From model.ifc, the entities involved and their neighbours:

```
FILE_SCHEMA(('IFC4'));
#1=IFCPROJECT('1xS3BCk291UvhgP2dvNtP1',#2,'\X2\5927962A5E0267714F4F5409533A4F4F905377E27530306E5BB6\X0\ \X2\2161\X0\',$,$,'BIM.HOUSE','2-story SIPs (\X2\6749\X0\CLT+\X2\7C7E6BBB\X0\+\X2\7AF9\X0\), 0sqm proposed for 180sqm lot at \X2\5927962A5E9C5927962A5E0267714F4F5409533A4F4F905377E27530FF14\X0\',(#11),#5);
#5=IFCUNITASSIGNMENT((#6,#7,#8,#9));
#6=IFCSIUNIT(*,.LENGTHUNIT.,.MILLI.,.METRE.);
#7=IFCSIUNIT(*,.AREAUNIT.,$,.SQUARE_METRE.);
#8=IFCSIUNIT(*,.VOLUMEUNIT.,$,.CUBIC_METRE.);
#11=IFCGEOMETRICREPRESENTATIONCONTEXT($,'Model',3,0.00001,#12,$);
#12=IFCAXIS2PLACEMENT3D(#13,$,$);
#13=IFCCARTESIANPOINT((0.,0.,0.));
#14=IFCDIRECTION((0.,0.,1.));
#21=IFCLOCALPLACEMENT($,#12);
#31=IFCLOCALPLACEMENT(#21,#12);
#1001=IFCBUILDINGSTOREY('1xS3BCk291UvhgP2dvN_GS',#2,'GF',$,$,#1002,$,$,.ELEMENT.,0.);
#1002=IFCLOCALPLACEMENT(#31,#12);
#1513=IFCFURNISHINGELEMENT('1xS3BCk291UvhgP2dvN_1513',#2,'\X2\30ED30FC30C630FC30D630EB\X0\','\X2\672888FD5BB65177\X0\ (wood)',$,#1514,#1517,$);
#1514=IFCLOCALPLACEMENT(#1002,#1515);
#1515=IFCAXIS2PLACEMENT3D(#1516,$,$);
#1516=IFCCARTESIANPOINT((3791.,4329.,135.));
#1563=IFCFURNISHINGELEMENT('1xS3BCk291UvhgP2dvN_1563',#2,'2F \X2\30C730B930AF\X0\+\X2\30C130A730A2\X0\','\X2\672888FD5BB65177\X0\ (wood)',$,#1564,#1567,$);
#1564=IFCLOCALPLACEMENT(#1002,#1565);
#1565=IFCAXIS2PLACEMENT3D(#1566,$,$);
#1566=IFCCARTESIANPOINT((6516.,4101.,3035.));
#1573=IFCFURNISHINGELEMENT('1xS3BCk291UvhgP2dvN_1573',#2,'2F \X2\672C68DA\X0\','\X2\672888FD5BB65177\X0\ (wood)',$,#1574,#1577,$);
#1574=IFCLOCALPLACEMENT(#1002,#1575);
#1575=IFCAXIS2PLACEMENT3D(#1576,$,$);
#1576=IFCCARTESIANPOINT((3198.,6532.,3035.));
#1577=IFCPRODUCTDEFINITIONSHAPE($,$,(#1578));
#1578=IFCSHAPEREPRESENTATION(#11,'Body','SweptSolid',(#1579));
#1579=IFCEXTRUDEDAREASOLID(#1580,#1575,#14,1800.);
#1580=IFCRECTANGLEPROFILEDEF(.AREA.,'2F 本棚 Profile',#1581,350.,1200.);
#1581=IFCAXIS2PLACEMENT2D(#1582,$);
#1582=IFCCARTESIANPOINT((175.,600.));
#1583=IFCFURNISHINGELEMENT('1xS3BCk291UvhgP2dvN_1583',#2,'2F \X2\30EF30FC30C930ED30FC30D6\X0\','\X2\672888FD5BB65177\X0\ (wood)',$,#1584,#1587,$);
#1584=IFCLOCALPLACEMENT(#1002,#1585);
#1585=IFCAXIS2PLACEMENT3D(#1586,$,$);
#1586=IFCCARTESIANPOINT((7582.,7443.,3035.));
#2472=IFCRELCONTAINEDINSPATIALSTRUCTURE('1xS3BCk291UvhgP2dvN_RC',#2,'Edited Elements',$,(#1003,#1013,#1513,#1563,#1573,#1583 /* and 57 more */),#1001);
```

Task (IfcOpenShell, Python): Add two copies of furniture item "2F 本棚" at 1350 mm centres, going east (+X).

```python
import numpy as np
import ifcopenshell
import ifcopenshell.api.geometry
import ifcopenshell.api.root
import ifcopenshell.util.element
import ifcopenshell.util.placement

model = ifcopenshell.open("model.ifc")


def reuse_history(source, copy):
    """copy_class also copies each property set's owner history, people and application; keep the originals."""
    for rel in copy.IsDefinedBy:
        if rel.is_a("IfcRelDefinesByProperties") and (history := rel.RelatingPropertyDefinition.OwnerHistory):
            rel.RelatingPropertyDefinition.OwnerHistory = source.OwnerHistory
            ifcopenshell.util.element.remove_deep2(model, history)


source = model.by_guid("1xS3BCk291UvhgP2dvN_1573")
base = ifcopenshell.util.placement.get_local_placement(source.ObjectPlacement)
step = np.array([1.0, 0.0, 0.0]) * 1350.0

for i in range(1, 3):
    copy = ifcopenshell.api.root.copy_class(model, product=source)
    copy.Representation = ifcopenshell.util.element.copy_deep(
        model, source.Representation, exclude=["IfcGeometricRepresentationContext", "IfcRepresentationMap"]
    )
    reuse_history(source, copy)
    matrix = base.copy()
    matrix[:3, 3] += i * step
    print("added at", matrix[:3, 3].round(3) + 0.0)
    ifcopenshell.api.geometry.edit_object_placement(model, product=copy, matrix=matrix, is_si=False)

model.write("model_updated.ifc")
```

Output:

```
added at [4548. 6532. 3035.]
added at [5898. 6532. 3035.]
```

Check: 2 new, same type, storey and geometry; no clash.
